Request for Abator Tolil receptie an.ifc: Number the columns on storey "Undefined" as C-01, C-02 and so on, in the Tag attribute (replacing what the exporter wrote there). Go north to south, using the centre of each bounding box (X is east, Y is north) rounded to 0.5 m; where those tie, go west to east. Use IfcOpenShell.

First a look at what the model holds.

```python
import ifcopenshell
import ifcopenshell.util.element
import ifcopenshell.util.placement

model = ifcopenshell.open("Abator Tolil receptie an.ifc")
print(model.schema)
storey = next(s for s in model.by_type("IfcBuildingStorey") if s.Name == "Undefined")
columns = [e for e in ifcopenshell.util.element.get_decomposition(storey) if e.is_a("IfcColumn")]
for e in sorted(columns, key=lambda e: e.id()):
    origin = ifcopenshell.util.placement.get_local_placement(e.ObjectPlacement)[:3, 3]
    print(e.id(), e.Tag, e.Name, origin.round(2) + 0.0, sep=" | ")
```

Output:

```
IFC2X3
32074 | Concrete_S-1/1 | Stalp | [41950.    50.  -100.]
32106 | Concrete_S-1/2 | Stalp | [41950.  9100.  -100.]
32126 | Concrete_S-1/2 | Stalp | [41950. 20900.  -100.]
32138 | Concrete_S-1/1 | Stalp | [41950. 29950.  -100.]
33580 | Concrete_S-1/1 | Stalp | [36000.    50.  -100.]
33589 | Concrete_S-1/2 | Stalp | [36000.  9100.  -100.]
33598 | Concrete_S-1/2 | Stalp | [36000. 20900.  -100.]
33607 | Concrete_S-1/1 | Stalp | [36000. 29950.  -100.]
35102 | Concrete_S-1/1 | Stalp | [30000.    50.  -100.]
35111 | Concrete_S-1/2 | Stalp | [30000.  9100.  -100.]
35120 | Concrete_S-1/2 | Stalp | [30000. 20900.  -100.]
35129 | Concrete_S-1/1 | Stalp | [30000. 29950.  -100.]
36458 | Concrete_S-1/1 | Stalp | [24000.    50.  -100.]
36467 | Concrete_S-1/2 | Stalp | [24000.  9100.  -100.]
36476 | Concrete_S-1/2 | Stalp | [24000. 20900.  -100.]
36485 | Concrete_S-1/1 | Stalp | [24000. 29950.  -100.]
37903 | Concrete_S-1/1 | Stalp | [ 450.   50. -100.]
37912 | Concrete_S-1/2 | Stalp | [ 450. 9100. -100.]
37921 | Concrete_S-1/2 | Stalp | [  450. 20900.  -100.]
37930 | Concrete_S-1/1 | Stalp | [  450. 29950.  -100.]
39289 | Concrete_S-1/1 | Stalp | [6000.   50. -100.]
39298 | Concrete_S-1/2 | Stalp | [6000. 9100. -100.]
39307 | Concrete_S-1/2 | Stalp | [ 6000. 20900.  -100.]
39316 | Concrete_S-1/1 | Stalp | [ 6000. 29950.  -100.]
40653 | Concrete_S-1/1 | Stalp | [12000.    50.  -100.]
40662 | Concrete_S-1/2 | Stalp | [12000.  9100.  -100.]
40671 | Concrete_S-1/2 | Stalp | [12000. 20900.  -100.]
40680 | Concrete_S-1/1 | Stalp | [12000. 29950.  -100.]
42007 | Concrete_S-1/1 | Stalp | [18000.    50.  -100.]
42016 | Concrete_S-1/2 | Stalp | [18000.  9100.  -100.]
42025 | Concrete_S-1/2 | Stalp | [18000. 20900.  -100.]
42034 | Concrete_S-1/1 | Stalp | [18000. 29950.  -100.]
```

```python
import ifcopenshell
import ifcopenshell.geom
import ifcopenshell.util.element
import ifcopenshell.util.shape

model = ifcopenshell.open("Abator Tolil receptie an.ifc")
settings = ifcopenshell.geom.settings()
settings.set("use-world-coords", True)


def centre(element):
    shape = ifcopenshell.geom.create_shape(settings, element)
    return ifcopenshell.util.shape.get_bbox_centroid(shape.geometry)


storey = next(s for s in model.by_type("IfcBuildingStorey") if s.Name == "Undefined")
columns = [e for e in ifcopenshell.util.element.get_decomposition(storey) if e.is_a("IfcColumn")]

# Insertion points can sit at a corner or the storey origin, so sort by the geometry (in metres).
centres = {e: centre(e) for e in columns}
columns.sort(key=lambda e: (-round(centres[e][1] / 0.5), centres[e][0]))

for i, e in enumerate(columns, start=1):
    number = f"C-{i:02d}"
    e.Tag = number
    print(e.id(), number)

model.write("Abator Tolil receptie an-out.ifc")
```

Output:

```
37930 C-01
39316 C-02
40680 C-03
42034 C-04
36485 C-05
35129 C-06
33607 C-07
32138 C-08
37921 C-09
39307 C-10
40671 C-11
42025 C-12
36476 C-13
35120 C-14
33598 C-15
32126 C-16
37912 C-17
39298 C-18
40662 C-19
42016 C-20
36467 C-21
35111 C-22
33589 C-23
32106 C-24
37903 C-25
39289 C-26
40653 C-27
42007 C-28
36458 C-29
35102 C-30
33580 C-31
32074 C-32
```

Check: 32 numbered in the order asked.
